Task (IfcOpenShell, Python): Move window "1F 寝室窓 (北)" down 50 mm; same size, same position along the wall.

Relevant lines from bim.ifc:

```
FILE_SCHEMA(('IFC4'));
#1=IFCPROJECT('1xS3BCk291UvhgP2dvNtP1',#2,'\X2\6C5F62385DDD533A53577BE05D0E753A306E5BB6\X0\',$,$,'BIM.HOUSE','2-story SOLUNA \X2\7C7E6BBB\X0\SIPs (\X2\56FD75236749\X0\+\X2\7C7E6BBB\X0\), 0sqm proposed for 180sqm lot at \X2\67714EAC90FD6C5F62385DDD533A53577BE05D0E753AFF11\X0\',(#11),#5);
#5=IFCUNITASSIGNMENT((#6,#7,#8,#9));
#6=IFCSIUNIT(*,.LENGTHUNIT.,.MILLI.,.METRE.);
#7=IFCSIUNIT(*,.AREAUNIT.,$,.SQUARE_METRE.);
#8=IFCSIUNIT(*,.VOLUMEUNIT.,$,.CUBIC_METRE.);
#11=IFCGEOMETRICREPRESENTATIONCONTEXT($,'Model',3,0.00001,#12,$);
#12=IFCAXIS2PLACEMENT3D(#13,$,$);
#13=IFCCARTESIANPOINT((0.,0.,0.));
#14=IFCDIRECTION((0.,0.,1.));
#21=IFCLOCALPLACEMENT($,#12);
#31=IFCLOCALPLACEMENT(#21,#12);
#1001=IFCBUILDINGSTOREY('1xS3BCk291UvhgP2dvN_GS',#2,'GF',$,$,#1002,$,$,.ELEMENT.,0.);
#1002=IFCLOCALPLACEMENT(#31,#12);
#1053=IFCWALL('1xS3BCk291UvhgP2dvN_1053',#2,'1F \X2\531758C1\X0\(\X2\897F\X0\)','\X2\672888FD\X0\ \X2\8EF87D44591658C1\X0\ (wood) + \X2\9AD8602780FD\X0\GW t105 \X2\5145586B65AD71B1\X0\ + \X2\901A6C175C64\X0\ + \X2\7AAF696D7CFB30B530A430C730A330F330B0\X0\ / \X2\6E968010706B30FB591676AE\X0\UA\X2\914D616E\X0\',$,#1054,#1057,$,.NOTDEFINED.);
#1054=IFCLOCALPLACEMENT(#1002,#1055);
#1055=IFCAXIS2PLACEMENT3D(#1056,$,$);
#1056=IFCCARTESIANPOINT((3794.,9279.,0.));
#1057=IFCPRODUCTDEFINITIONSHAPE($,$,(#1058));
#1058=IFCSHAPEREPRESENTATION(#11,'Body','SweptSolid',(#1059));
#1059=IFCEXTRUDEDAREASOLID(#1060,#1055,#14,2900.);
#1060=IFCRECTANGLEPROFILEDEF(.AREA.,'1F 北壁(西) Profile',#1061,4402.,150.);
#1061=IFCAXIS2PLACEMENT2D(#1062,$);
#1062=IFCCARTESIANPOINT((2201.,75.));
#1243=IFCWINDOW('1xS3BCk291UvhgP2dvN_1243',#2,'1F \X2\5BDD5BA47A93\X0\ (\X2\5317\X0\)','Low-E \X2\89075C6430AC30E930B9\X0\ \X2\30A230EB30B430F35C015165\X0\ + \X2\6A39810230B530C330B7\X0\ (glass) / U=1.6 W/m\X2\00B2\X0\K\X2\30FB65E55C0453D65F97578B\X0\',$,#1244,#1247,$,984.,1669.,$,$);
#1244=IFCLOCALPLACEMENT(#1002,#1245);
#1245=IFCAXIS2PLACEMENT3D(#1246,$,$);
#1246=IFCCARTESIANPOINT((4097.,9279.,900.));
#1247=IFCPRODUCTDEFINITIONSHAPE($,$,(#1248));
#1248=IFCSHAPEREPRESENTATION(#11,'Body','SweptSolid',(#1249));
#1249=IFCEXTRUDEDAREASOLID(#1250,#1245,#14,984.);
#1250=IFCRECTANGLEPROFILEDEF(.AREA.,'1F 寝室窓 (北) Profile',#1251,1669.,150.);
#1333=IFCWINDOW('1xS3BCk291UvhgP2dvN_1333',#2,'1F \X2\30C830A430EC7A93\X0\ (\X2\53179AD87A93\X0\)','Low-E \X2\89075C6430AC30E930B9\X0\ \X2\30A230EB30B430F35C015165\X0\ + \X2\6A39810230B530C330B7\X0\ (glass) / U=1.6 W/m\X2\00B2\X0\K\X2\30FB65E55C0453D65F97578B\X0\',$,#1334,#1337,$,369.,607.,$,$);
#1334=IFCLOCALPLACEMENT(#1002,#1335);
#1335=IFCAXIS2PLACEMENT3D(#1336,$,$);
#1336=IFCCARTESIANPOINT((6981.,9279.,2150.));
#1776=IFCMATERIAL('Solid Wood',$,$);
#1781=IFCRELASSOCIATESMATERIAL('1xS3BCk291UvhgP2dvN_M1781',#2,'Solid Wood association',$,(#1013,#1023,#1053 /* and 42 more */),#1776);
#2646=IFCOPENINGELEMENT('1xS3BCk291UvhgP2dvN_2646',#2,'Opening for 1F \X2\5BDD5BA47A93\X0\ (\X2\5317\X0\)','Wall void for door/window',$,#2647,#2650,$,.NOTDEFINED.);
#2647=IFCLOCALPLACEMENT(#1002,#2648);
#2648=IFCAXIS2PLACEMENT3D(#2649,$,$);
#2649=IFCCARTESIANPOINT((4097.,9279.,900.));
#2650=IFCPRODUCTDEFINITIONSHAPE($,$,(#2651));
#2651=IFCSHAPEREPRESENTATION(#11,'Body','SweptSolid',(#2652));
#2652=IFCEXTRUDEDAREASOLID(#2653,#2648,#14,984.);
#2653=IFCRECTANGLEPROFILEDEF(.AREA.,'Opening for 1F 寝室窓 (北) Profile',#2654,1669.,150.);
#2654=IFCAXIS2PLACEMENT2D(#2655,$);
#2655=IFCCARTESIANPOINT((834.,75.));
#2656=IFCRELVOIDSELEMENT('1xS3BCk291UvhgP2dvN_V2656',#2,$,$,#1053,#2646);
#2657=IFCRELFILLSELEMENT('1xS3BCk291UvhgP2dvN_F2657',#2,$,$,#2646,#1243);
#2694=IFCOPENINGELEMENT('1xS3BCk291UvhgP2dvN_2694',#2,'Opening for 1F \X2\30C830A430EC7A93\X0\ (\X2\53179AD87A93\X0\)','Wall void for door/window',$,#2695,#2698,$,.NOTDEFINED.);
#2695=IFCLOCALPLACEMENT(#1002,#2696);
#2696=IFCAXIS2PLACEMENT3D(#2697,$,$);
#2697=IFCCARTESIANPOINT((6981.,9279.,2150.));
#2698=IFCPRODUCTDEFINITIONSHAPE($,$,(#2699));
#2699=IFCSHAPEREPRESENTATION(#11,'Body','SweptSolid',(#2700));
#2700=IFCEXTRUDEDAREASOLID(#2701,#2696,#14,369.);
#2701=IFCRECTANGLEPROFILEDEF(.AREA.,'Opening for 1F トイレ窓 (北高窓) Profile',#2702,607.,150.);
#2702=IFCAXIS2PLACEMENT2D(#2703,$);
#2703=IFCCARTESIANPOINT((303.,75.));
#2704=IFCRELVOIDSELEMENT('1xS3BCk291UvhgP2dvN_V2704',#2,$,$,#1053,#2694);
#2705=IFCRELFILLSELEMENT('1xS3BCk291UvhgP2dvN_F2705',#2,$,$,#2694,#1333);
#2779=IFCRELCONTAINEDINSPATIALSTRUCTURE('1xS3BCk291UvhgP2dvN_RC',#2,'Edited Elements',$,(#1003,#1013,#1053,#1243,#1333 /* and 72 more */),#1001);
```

```python
import numpy as np
import ifcopenshell
import ifcopenshell.api.geometry
import ifcopenshell.util.placement
import ifcopenshell.util.unit

model = ifcopenshell.open("bim.ifc")
unit_scale = ifcopenshell.util.unit.calculate_unit_scale(model)

window = model.by_id(1243)
opening = window.FillsVoids[0].RelatingOpeningElement
dz = -0.05 / unit_scale

shift = np.array([0.0, 0.0, dz])
# The window is not placed relative to its opening, so move both.
for product in (opening, window):
    matrix = ifcopenshell.util.placement.get_local_placement(product.ObjectPlacement)
    matrix[:3, 3] += shift
    ifcopenshell.api.geometry.edit_object_placement(model, product=product, matrix=matrix, is_si=False)

print(f"moved by {dz * unit_scale:+.3f} m")

model.write("bim_updated.ifc")
```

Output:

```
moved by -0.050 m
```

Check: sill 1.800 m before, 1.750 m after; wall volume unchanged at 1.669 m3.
